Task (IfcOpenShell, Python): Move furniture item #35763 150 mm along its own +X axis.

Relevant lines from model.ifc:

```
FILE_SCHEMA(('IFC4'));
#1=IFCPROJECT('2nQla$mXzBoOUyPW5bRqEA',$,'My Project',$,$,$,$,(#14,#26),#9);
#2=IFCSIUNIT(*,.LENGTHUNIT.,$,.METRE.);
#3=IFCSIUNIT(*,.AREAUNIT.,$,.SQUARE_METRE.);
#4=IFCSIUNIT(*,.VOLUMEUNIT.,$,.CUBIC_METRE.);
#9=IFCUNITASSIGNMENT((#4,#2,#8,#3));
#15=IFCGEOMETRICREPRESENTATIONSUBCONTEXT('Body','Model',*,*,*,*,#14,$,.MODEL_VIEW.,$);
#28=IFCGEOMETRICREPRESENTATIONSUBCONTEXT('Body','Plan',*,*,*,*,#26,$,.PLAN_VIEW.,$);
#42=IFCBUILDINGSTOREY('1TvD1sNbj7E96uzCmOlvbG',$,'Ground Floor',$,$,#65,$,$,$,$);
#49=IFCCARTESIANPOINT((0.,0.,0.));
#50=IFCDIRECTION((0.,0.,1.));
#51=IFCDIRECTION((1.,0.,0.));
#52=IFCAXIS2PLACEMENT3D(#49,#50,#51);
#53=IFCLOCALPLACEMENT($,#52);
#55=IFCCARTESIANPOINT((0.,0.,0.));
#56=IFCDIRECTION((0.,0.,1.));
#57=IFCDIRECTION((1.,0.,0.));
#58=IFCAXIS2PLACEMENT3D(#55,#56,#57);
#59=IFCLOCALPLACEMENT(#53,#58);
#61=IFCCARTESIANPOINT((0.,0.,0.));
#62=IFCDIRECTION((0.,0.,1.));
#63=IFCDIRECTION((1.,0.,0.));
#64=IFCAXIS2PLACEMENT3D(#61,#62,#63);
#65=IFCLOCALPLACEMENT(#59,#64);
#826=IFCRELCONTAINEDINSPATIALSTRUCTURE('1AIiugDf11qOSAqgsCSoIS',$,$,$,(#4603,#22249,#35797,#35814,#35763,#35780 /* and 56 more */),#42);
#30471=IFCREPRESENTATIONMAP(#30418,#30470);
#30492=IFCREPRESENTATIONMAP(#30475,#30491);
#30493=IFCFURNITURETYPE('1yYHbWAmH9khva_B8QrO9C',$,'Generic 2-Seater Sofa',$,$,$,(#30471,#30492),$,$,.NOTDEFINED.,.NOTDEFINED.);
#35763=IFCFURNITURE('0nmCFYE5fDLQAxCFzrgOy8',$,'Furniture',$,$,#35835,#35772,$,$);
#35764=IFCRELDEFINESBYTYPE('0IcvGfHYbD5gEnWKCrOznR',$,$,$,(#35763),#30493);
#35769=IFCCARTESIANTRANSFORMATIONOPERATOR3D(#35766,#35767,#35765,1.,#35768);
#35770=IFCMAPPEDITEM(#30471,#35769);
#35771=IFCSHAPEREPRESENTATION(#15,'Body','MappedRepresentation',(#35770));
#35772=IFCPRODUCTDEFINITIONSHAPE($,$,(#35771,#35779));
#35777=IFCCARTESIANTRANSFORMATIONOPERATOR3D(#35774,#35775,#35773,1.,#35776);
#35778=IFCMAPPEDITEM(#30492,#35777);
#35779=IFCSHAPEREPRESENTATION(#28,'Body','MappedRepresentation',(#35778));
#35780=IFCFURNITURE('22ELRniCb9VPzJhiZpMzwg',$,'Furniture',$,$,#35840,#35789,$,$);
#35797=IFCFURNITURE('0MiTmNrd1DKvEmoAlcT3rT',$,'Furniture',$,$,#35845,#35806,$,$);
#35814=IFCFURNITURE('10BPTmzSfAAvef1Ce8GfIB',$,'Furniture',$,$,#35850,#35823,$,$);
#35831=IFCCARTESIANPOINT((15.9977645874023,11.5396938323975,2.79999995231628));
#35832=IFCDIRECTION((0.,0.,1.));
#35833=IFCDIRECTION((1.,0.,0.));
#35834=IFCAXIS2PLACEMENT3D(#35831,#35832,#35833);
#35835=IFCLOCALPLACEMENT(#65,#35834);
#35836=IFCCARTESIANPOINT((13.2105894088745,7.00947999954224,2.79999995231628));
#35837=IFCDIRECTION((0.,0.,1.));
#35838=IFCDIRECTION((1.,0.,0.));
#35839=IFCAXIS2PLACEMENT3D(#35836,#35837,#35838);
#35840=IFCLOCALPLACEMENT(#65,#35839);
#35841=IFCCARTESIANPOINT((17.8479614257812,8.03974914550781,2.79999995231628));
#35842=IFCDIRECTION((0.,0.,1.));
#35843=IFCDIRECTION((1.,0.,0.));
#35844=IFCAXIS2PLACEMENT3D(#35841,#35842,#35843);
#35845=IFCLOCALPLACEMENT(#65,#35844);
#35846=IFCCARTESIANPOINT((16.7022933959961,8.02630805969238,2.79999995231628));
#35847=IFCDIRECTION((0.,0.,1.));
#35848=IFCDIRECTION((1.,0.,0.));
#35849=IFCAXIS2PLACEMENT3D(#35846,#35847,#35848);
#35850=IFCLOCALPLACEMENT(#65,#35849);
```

```python
import ifcopenshell
import ifcopenshell.api.geometry
import ifcopenshell.util.placement
import ifcopenshell.util.unit

model = ifcopenshell.open("model.ifc")
unit_scale = ifcopenshell.util.unit.calculate_unit_scale(model)

item = model.by_guid("0nmCFYE5fDLQAxCFzrgOy8")
matrix = ifcopenshell.util.placement.get_local_placement(item.ObjectPlacement)
matrix[:3, 3] += matrix[:3, 0] * 0.15 / unit_scale
ifcopenshell.api.geometry.edit_object_placement(model, product=item, matrix=matrix, is_si=False)

print(ifcopenshell.util.placement.get_local_placement(item.ObjectPlacement).round(3) + 0.0)

model.write("model_rev.ifc")
```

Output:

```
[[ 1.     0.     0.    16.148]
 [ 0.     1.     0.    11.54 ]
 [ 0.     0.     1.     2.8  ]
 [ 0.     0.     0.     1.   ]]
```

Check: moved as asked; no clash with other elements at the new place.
